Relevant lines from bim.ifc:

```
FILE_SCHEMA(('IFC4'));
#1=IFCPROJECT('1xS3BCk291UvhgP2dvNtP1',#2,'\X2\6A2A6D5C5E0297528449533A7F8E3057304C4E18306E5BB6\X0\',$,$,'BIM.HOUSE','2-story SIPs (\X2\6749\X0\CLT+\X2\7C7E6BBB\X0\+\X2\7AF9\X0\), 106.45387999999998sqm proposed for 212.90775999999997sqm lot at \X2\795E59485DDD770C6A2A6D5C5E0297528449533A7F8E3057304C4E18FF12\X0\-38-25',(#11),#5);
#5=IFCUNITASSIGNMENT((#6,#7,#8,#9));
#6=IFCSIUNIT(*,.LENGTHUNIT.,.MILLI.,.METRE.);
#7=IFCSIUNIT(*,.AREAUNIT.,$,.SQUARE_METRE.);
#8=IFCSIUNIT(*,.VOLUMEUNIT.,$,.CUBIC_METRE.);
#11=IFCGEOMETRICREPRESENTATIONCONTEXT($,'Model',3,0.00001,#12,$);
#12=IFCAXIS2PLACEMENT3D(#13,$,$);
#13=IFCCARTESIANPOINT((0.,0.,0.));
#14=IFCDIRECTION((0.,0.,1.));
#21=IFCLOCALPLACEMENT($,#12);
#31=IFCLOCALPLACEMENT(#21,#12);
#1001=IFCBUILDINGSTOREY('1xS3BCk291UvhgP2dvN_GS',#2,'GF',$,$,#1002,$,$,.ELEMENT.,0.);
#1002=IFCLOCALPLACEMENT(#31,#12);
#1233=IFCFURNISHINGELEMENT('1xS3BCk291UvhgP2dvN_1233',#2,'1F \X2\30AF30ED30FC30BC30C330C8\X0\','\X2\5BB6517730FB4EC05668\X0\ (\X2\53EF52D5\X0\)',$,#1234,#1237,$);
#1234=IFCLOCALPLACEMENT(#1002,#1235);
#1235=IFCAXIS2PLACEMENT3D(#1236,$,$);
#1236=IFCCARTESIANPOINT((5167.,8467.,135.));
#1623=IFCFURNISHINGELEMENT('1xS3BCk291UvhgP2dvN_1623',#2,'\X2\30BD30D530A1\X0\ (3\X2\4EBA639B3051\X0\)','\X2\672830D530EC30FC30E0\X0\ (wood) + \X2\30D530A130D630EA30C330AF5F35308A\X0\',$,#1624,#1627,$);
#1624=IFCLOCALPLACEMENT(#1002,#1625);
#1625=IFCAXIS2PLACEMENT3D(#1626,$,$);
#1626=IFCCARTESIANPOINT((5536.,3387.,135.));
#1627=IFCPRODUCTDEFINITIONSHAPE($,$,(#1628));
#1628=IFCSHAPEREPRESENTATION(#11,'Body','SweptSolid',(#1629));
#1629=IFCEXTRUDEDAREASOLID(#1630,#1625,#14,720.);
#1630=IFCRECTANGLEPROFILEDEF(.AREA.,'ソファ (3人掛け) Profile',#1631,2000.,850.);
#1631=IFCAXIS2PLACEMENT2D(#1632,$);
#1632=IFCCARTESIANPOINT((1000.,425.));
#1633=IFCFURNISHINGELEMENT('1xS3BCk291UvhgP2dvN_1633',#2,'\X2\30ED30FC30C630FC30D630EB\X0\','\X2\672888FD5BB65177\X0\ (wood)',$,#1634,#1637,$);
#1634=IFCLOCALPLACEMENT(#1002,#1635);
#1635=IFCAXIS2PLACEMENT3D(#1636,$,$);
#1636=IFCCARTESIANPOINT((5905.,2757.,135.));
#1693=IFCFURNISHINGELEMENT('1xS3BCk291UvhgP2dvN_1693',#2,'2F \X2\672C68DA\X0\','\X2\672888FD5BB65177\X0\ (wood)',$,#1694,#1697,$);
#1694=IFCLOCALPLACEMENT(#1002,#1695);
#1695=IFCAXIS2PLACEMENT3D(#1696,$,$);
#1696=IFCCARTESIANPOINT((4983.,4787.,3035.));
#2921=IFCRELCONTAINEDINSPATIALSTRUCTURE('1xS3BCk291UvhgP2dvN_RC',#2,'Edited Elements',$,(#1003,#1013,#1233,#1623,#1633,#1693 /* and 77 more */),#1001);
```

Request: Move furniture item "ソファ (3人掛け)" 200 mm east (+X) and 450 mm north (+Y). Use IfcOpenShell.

```python
import ifcopenshell
import ifcopenshell.api.geometry
import ifcopenshell.util.placement
import ifcopenshell.util.unit

model = ifcopenshell.open("bim.ifc")
unit_scale = ifcopenshell.util.unit.calculate_unit_scale(model)

item = model.by_guid("1xS3BCk291UvhgP2dvN_1623")
matrix = ifcopenshell.util.placement.get_local_placement(item.ObjectPlacement)
matrix[0, 3] += 0.2 / unit_scale
matrix[1, 3] += 0.45 / unit_scale
ifcopenshell.api.geometry.edit_object_placement(model, product=item, matrix=matrix, is_si=False)

print(ifcopenshell.util.placement.get_local_placement(item.ObjectPlacement).round(3) + 0.0)

model.write("bim-out.ifc")
```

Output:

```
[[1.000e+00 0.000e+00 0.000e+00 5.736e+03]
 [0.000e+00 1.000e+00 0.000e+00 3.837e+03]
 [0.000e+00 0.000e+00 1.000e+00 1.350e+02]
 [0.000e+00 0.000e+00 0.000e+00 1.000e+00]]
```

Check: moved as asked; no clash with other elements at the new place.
